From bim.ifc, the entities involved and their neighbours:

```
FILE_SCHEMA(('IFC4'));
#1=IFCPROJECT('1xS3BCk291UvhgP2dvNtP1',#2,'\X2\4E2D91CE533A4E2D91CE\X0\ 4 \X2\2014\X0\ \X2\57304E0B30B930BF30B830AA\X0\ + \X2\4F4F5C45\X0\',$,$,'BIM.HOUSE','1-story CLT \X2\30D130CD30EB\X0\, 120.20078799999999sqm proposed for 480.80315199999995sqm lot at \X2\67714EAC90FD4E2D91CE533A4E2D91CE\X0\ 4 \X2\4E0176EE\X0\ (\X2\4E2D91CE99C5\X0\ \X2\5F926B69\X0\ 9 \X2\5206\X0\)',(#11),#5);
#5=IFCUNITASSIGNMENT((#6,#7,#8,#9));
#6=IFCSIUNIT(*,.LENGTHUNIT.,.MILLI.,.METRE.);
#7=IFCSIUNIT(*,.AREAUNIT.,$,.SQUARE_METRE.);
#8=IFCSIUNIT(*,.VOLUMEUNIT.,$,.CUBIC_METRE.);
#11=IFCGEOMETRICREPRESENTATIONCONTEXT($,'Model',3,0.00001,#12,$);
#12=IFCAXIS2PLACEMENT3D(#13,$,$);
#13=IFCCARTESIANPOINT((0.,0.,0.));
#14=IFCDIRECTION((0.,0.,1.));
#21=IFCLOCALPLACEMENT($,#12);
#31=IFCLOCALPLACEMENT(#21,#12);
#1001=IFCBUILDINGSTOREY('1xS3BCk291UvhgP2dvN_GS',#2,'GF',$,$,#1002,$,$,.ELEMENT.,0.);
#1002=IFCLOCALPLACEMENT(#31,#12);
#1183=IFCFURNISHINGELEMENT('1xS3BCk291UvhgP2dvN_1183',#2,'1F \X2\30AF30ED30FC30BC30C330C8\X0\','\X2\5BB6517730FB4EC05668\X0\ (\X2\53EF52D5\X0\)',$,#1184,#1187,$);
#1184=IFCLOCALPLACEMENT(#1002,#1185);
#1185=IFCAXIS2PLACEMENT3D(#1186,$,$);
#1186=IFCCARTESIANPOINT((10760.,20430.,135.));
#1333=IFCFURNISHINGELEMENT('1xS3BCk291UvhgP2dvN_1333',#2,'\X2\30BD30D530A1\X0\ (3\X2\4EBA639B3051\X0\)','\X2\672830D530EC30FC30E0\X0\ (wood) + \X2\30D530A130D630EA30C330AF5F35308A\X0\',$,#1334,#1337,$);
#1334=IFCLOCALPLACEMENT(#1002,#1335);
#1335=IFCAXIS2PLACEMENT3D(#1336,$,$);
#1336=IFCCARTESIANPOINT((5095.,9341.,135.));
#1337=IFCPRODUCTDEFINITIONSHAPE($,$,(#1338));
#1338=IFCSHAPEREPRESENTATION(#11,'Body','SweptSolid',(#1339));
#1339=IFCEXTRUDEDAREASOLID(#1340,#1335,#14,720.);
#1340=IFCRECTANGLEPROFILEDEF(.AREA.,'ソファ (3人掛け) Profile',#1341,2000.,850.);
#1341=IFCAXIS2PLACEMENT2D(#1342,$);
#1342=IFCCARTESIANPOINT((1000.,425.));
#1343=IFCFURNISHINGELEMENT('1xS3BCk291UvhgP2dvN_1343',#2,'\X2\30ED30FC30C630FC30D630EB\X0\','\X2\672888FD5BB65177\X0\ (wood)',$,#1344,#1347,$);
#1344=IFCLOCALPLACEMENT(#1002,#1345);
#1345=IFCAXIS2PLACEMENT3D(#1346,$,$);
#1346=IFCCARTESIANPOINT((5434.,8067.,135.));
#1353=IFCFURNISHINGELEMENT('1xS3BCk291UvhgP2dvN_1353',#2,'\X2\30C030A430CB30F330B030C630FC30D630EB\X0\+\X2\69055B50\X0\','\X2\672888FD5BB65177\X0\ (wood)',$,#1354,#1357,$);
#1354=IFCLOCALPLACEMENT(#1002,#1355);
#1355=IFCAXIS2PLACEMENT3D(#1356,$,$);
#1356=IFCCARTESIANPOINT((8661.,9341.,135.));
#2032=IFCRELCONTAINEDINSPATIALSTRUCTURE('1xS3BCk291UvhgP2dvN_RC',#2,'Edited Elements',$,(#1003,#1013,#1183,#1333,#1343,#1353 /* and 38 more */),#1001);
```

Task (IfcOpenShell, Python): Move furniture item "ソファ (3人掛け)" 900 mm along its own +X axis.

```python
import ifcopenshell
import ifcopenshell.api.geometry
import ifcopenshell.util.placement

model = ifcopenshell.open("bim.ifc")

item = model.by_guid("1xS3BCk291UvhgP2dvN_1333")
matrix = ifcopenshell.util.placement.get_local_placement(item.ObjectPlacement)
matrix[:3, 3] += matrix[:3, 0] * 900.0
ifcopenshell.api.geometry.edit_object_placement(model, product=item, matrix=matrix, is_si=False)

print(ifcopenshell.util.placement.get_local_placement(item.ObjectPlacement).round(3) + 0.0)

model.write("bim_updated.ifc")
```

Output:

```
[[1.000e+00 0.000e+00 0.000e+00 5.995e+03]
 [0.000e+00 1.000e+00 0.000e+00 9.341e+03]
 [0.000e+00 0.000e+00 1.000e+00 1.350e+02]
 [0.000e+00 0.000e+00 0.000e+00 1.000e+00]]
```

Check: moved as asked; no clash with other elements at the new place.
